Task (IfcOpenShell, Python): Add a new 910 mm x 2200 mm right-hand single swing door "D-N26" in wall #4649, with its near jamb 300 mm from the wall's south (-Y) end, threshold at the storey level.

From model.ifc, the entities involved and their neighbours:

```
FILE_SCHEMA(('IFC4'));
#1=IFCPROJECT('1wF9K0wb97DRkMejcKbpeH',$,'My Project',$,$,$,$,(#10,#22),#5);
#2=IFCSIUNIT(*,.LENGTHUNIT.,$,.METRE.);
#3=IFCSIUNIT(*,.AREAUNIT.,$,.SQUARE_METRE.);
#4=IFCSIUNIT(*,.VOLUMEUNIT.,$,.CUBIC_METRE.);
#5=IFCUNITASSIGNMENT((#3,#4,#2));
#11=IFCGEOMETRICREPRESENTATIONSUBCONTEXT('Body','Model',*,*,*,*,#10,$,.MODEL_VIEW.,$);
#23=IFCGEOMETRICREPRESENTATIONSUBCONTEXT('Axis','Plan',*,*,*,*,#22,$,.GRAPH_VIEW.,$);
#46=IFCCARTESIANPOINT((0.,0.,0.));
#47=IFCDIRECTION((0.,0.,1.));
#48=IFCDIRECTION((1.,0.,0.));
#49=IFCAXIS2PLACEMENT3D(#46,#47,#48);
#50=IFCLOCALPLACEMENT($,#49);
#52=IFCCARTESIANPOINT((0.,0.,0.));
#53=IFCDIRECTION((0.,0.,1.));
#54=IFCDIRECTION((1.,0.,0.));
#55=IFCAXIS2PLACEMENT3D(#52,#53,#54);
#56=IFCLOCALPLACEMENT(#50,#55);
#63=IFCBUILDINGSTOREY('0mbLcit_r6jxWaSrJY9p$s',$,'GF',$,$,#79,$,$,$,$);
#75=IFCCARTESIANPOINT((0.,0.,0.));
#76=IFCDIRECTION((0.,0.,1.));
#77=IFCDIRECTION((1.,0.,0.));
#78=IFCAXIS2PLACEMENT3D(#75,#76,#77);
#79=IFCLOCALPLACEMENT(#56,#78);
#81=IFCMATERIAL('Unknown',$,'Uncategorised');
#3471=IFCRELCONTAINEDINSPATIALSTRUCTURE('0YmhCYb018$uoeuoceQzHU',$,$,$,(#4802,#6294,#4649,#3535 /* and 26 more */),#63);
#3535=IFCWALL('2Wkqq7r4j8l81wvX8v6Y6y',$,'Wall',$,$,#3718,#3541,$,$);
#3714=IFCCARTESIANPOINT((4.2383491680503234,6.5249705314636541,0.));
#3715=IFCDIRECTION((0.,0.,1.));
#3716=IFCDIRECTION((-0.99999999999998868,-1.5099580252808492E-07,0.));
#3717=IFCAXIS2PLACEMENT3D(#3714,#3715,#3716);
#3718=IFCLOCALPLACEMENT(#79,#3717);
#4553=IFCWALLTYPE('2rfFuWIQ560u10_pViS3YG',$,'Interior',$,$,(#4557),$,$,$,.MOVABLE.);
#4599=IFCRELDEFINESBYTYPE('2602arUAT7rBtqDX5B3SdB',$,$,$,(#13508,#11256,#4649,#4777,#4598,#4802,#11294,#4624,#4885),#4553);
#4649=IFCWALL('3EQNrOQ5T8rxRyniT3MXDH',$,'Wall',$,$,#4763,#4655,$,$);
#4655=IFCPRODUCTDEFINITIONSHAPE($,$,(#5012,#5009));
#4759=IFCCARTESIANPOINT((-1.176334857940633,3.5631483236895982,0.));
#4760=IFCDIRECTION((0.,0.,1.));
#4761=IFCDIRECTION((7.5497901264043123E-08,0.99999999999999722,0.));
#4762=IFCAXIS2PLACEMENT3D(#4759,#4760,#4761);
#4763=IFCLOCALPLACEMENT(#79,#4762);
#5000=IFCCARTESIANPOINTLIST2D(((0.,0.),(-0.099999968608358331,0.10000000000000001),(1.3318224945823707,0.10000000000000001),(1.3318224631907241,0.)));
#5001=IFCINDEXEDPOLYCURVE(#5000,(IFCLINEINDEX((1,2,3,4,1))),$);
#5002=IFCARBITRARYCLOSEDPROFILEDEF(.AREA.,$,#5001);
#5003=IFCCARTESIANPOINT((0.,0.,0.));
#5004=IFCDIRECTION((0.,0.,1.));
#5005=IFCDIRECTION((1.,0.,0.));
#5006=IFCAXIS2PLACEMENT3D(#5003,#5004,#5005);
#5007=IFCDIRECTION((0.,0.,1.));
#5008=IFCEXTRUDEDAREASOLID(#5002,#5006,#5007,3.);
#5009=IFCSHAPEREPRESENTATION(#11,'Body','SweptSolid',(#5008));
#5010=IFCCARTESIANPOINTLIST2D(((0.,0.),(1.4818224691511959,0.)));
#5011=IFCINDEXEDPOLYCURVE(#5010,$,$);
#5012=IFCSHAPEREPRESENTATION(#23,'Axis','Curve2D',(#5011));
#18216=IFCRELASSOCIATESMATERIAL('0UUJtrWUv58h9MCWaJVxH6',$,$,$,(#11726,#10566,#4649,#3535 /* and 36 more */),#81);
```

```python
import numpy as np
import ifcopenshell
import ifcopenshell.api.feature
import ifcopenshell.api.geometry
import ifcopenshell.api.root
import ifcopenshell.api.spatial
import ifcopenshell.geom
import ifcopenshell.util.element
import ifcopenshell.util.placement
import ifcopenshell.util.representation
import ifcopenshell.util.shape
import ifcopenshell.util.unit

model = ifcopenshell.open("model.ifc")
unit_scale = ifcopenshell.util.unit.calculate_unit_scale(model)
settings = ifcopenshell.geom.settings()


def volume(element):
    """Net volume in cubic metres, openings subtracted."""
    shape = ifcopenshell.geom.create_shape(settings, element)
    return ifcopenshell.util.shape.get_volume(shape.geometry)


wall = model.by_guid("3EQNrOQ5T8rxRyniT3MXDH")
storey = ifcopenshell.util.element.get_container(wall, ifc_class="IfcBuildingStorey")
context = ifcopenshell.util.representation.get_context(model, "Model", "Body", "MODEL_VIEW")
before = volume(wall)

width, height, from_end, sill = 0.91, 2.2, 0.3, 0.0  # metres

# The wall runs along its own X axis, and the end named is its -X end.
wall_shape = ifcopenshell.geom.create_shape(settings, wall)
x, y, z = ifcopenshell.util.shape.get_vertices(wall_shape.geometry).T
start = x.min() + from_end
face, thickness = float(y.min()), float(y.max() - y.min())
wall_matrix = ifcopenshell.util.placement.get_local_placement(wall.ObjectPlacement)
level = ifcopenshell.util.placement.get_local_placement(storey.ObjectPlacement)[2, 3]


def in_wall(x, y):
    """Placement at x, y metres in the wall's axes, at sill height."""
    matrix = wall_matrix.copy()
    matrix[:, 3] = wall_matrix @ np.array([x / unit_scale, y / unit_scale, 0.0, 1.0])
    matrix[2, 3] = level + sill / unit_scale
    return matrix


# Opening: a box that overshoots both wall faces by 50 mm.
opening = ifcopenshell.api.root.create_entity(model, ifc_class="IfcOpeningElement", predefined_type="OPENING")
box = ifcopenshell.api.geometry.add_wall_representation(
    model, context=context, length=width, height=height, thickness=thickness + 0.1
)
ifcopenshell.api.geometry.assign_representation(model, product=opening, representation=box)
ifcopenshell.api.geometry.edit_object_placement(model, product=opening, matrix=in_wall(start, face - 0.05), is_si=False)
ifcopenshell.api.feature.add_feature(model, feature=opening, element=wall)

door = ifcopenshell.api.root.create_entity(model, ifc_class="IfcDoor", name="D-N26", predefined_type="DOOR")
door.OverallWidth, door.OverallHeight = width / unit_scale, height / unit_scale
door.OperationType = "SINGLE_SWING_RIGHT"
body = ifcopenshell.api.geometry.add_door_representation(
    model,
    context=context,
    overall_width=door.OverallWidth,
    overall_height=door.OverallHeight,
    operation_type="SINGLE_SWING_RIGHT",
    lining_properties={"LiningDepth": thickness / unit_scale, "ThresholdDepth": thickness / unit_scale},
)
ifcopenshell.api.geometry.assign_representation(model, product=door, representation=body)
ifcopenshell.api.spatial.assign_container(model, products=[door], relating_structure=storey)
ifcopenshell.api.feature.add_filling(model, opening=opening, element=door)

# The lining spans the wall, so the door starts at the wall face.
ifcopenshell.api.geometry.edit_object_placement(model, product=door, matrix=in_wall(start, face), is_si=False)

after = volume(wall)

print(f"wall volume {before:.3f} -> {after:.3f} m3")

model.write("model_edited.ifc")
```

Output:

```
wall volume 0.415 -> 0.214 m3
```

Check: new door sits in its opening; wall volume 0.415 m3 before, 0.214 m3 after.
